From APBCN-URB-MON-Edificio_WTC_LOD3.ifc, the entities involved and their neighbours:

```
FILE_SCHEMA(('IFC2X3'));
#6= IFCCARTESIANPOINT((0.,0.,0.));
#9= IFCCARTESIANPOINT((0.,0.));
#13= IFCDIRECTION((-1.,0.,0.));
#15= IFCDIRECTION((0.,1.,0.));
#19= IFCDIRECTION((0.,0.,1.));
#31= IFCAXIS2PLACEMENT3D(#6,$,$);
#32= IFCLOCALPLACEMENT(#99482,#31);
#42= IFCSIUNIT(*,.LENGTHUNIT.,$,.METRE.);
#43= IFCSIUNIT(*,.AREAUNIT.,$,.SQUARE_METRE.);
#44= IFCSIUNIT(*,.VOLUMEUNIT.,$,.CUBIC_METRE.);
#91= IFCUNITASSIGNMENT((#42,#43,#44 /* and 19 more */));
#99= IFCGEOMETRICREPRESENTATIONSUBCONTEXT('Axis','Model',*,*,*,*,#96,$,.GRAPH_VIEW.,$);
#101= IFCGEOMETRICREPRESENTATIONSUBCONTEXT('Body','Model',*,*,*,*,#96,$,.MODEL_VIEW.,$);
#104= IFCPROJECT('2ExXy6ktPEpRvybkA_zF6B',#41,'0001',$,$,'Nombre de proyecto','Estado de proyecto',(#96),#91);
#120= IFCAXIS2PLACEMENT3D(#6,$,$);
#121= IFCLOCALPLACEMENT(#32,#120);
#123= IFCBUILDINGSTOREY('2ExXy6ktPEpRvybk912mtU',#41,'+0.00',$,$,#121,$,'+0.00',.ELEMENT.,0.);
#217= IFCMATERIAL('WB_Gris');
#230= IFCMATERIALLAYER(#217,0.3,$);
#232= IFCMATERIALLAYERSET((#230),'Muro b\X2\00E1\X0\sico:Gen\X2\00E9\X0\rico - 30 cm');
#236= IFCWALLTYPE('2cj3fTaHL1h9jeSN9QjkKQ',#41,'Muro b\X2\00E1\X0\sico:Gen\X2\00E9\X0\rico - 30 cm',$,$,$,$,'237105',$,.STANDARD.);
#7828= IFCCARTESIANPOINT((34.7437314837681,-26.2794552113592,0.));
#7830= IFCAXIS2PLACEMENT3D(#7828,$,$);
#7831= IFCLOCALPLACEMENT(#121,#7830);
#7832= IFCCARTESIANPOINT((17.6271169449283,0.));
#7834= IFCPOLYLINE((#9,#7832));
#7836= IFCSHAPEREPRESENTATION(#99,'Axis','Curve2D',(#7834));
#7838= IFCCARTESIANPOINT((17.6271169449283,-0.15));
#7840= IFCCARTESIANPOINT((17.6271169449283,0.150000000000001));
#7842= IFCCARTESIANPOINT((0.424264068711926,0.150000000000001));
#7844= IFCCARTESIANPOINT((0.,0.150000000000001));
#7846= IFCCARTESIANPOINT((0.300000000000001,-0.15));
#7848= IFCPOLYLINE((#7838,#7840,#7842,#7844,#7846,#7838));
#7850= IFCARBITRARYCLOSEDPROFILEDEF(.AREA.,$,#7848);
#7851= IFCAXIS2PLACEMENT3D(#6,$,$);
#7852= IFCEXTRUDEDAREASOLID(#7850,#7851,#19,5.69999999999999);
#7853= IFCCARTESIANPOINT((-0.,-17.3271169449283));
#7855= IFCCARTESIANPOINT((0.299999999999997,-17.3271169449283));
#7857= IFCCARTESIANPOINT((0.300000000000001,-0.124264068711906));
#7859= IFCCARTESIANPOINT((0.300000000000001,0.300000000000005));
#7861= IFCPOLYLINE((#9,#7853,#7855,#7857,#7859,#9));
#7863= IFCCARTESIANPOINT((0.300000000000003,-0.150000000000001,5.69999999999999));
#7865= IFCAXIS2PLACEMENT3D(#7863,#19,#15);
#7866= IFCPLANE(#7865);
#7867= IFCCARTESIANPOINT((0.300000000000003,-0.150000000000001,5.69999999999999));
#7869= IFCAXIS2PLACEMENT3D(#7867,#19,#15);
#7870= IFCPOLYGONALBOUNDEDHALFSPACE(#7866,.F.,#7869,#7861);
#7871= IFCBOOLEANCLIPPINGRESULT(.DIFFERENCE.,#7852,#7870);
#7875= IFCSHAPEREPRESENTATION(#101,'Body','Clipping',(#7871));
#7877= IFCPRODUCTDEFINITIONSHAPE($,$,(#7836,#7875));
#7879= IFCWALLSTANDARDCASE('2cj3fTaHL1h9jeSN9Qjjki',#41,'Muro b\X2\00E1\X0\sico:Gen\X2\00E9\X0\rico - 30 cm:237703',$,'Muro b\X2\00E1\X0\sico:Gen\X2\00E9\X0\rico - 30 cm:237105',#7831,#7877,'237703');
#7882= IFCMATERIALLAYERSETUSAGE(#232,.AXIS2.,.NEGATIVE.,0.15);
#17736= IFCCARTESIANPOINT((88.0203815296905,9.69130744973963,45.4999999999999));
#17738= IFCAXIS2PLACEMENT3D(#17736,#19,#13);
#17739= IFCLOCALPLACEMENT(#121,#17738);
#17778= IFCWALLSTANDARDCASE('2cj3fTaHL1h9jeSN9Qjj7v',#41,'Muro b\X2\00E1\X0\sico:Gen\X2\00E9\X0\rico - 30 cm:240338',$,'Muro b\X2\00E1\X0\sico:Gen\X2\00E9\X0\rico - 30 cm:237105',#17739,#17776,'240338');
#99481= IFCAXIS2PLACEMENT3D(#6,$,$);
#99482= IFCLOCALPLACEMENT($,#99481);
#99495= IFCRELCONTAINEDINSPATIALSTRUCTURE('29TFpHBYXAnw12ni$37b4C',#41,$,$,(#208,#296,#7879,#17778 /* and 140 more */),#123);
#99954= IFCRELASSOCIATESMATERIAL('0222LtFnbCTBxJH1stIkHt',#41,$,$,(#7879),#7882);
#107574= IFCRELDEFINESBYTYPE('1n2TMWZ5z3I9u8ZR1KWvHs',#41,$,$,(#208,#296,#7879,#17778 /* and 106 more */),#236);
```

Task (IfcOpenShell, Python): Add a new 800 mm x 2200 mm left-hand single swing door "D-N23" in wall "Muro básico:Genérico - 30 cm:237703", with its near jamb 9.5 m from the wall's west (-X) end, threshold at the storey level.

```python
import numpy as np
import ifcopenshell
import ifcopenshell.api.feature
import ifcopenshell.api.geometry
import ifcopenshell.api.root
import ifcopenshell.api.spatial
import ifcopenshell.api.type
import ifcopenshell.geom
import ifcopenshell.util.element
import ifcopenshell.util.placement
import ifcopenshell.util.representation
import ifcopenshell.util.shape
import ifcopenshell.util.unit

model = ifcopenshell.open("APBCN-URB-MON-Edificio_WTC_LOD3.ifc")
unit_scale = ifcopenshell.util.unit.calculate_unit_scale(model)
settings = ifcopenshell.geom.settings()


def volume(element):
    """Net volume in cubic metres, openings subtracted."""
    shape = ifcopenshell.geom.create_shape(settings, element)
    return ifcopenshell.util.shape.get_volume(shape.geometry)


wall = model.by_guid("2cj3fTaHL1h9jeSN9Qjjki")
storey = ifcopenshell.util.element.get_container(wall, ifc_class="IfcBuildingStorey")
context = ifcopenshell.util.representation.get_context(model, "Model", "Body", "MODEL_VIEW")
before = volume(wall)

width, height, from_end, sill = 0.8, 2.2, 9.5, 0.0  # metres

# The wall runs along its own X axis, and the end named is its -X end.
wall_shape = ifcopenshell.geom.create_shape(settings, wall)
x, y, z = ifcopenshell.util.shape.get_vertices(wall_shape.geometry).T
start = x.min() + from_end
face, thickness = float(y.min()), float(y.max() - y.min())
wall_matrix = ifcopenshell.util.placement.get_local_placement(wall.ObjectPlacement)
level = ifcopenshell.util.placement.get_local_placement(storey.ObjectPlacement)[2, 3]


def in_wall(x, y):
    """Placement at x, y metres in the wall's axes, at sill height."""
    matrix = wall_matrix.copy()
    matrix[:, 3] = wall_matrix @ np.array([x / unit_scale, y / unit_scale, 0.0, 1.0])
    matrix[2, 3] = level + sill / unit_scale
    return matrix


# Opening: a box that overshoots both wall faces by 50 mm.
opening = ifcopenshell.api.root.create_entity(model, ifc_class="IfcOpeningElement")
box = ifcopenshell.api.geometry.add_wall_representation(
    model, context=context, length=width, height=height, thickness=thickness + 0.1
)
ifcopenshell.api.geometry.assign_representation(model, product=opening, representation=box)
ifcopenshell.api.geometry.edit_object_placement(model, product=opening, matrix=in_wall(start, face - 0.05), is_si=False)
ifcopenshell.api.feature.add_feature(model, feature=opening, element=wall)

door = ifcopenshell.api.root.create_entity(model, ifc_class="IfcDoor", name="D-N23")
door.OverallWidth, door.OverallHeight = width / unit_scale, height / unit_scale
body = ifcopenshell.api.geometry.add_door_representation(
    model,
    context=context,
    overall_width=door.OverallWidth,
    overall_height=door.OverallHeight,
    operation_type="SINGLE_SWING_LEFT",
    lining_properties={"LiningDepth": thickness / unit_scale, "ThresholdDepth": thickness / unit_scale},
)
ifcopenshell.api.geometry.assign_representation(model, product=door, representation=body)
ifcopenshell.api.spatial.assign_container(model, products=[door], relating_structure=storey)
fills = ifcopenshell.api.feature.add_filling(model, opening=opening, element=door)
fills.OwnerHistory = door.OwnerHistory  # required in IFC2X3

# IFC2X3 keeps the operation on the door style.
style = ifcopenshell.api.root.create_entity(model, ifc_class="IfcDoorStyle", name="D-N23")
style.OperationType, style.ConstructionType = "SINGLE_SWING_LEFT", "NOTDEFINED"
style.ParameterTakesPrecedence = style.Sizeable = False
ifcopenshell.api.type.assign_type(model, related_objects=[door], relating_type=style)

# The lining spans the wall, so the door starts at the wall face.
ifcopenshell.api.geometry.edit_object_placement(model, product=door, matrix=in_wall(start, face), is_si=False)

after = volume(wall)

print(f"wall volume {before:.3f} -> {after:.3f} m3")

model.write("APBCN-URB-MON-Edificio_WTC_LOD3-out.ifc")
```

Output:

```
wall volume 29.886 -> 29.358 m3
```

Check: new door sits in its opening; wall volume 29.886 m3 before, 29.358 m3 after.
